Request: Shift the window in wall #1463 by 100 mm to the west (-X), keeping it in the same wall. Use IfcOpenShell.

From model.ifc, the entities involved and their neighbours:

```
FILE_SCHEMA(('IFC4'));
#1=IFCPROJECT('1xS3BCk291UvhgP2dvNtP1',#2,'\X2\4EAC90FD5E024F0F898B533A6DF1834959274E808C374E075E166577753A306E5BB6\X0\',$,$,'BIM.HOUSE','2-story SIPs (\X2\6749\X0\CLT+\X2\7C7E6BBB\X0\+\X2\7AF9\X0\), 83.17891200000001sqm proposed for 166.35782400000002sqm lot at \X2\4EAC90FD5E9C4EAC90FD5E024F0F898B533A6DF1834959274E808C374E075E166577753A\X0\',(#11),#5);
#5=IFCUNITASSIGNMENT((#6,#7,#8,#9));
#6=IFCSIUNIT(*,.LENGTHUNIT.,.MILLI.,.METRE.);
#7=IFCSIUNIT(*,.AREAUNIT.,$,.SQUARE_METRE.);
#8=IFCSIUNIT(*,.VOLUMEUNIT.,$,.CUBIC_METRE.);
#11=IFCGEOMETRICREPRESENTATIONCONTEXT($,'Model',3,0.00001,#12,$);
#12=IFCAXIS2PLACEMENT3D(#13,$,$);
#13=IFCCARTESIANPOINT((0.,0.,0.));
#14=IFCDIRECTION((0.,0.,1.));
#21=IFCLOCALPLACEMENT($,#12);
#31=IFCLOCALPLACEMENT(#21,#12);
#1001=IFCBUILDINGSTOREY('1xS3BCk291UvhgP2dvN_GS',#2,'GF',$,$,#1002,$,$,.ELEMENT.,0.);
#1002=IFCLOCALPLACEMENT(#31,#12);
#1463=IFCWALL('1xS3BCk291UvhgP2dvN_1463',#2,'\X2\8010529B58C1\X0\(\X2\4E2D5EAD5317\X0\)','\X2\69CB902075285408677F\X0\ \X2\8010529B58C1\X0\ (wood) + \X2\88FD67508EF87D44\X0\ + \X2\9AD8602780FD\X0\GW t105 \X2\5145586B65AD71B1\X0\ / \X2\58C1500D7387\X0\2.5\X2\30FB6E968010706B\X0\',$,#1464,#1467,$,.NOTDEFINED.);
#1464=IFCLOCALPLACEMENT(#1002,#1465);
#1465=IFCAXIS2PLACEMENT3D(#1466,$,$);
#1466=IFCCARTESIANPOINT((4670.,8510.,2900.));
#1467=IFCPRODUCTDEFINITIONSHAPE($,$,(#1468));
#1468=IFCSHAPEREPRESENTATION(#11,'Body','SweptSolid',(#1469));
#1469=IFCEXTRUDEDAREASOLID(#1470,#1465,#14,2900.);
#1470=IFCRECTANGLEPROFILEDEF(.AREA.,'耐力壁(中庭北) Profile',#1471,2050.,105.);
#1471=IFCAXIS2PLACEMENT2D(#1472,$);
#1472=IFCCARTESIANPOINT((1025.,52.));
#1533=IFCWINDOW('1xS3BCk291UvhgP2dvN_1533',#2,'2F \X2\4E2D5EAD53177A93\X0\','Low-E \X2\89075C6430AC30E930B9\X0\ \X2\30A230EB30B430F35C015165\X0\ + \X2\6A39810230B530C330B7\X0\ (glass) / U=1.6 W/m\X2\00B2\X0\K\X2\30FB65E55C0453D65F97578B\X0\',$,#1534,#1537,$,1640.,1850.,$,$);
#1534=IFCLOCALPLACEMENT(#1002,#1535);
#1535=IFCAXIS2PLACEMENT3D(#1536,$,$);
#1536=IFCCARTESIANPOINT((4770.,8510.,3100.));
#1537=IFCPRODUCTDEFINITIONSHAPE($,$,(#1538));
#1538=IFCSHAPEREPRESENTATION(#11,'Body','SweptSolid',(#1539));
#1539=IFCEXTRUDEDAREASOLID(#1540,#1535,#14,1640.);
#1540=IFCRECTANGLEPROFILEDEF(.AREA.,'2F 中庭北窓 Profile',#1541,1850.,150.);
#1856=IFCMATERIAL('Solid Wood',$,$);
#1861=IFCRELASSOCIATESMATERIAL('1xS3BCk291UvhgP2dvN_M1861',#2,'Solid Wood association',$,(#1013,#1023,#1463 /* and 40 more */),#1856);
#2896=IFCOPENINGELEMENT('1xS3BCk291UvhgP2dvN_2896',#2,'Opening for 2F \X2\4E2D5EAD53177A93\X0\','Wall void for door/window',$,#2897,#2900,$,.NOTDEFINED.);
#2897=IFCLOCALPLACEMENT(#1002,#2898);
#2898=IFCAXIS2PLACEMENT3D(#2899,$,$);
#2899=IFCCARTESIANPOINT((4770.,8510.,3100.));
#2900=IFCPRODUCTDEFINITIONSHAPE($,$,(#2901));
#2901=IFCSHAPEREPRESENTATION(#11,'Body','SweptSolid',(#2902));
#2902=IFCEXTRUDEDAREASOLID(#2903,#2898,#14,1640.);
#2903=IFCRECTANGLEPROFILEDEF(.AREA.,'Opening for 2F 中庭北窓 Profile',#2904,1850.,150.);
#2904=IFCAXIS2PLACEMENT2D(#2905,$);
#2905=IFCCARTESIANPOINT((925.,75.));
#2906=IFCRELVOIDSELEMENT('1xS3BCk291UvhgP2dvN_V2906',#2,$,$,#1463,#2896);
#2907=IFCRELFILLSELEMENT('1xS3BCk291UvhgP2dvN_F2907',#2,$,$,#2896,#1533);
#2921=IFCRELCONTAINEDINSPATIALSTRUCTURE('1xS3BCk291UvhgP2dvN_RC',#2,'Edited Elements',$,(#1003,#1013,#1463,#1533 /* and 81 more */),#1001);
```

```python
import ifcopenshell
import ifcopenshell.api.geometry
import ifcopenshell.util.placement
import ifcopenshell.util.unit

model = ifcopenshell.open("model.ifc")
unit_scale = ifcopenshell.util.unit.calculate_unit_scale(model)

window = model.by_guid("1xS3BCk291UvhgP2dvN_1533")
opening = window.FillsVoids[0].RelatingOpeningElement
wall = opening.VoidsElements[0].RelatingBuildingElement

wall_matrix = ifcopenshell.util.placement.get_local_placement(wall.ObjectPlacement)
shift = wall_matrix[:3, 0] * -0.1 / unit_scale
before = ifcopenshell.util.placement.get_local_placement(window.ObjectPlacement)[:3, 3].copy()

# The window is not placed relative to its opening, so move both.
for product in (opening, window):
    matrix = ifcopenshell.util.placement.get_local_placement(product.ObjectPlacement)
    matrix[:3, 3] += shift
    ifcopenshell.api.geometry.edit_object_placement(model, product=product, matrix=matrix, is_si=False)

after = ifcopenshell.util.placement.get_local_placement(window.ObjectPlacement)[:3, 3]
print("window moved by", (after - before).round(3) + 0.0)

model.write("model_v2.ifc")
```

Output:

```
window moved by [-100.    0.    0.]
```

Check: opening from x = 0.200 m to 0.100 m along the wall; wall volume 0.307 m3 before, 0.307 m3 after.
